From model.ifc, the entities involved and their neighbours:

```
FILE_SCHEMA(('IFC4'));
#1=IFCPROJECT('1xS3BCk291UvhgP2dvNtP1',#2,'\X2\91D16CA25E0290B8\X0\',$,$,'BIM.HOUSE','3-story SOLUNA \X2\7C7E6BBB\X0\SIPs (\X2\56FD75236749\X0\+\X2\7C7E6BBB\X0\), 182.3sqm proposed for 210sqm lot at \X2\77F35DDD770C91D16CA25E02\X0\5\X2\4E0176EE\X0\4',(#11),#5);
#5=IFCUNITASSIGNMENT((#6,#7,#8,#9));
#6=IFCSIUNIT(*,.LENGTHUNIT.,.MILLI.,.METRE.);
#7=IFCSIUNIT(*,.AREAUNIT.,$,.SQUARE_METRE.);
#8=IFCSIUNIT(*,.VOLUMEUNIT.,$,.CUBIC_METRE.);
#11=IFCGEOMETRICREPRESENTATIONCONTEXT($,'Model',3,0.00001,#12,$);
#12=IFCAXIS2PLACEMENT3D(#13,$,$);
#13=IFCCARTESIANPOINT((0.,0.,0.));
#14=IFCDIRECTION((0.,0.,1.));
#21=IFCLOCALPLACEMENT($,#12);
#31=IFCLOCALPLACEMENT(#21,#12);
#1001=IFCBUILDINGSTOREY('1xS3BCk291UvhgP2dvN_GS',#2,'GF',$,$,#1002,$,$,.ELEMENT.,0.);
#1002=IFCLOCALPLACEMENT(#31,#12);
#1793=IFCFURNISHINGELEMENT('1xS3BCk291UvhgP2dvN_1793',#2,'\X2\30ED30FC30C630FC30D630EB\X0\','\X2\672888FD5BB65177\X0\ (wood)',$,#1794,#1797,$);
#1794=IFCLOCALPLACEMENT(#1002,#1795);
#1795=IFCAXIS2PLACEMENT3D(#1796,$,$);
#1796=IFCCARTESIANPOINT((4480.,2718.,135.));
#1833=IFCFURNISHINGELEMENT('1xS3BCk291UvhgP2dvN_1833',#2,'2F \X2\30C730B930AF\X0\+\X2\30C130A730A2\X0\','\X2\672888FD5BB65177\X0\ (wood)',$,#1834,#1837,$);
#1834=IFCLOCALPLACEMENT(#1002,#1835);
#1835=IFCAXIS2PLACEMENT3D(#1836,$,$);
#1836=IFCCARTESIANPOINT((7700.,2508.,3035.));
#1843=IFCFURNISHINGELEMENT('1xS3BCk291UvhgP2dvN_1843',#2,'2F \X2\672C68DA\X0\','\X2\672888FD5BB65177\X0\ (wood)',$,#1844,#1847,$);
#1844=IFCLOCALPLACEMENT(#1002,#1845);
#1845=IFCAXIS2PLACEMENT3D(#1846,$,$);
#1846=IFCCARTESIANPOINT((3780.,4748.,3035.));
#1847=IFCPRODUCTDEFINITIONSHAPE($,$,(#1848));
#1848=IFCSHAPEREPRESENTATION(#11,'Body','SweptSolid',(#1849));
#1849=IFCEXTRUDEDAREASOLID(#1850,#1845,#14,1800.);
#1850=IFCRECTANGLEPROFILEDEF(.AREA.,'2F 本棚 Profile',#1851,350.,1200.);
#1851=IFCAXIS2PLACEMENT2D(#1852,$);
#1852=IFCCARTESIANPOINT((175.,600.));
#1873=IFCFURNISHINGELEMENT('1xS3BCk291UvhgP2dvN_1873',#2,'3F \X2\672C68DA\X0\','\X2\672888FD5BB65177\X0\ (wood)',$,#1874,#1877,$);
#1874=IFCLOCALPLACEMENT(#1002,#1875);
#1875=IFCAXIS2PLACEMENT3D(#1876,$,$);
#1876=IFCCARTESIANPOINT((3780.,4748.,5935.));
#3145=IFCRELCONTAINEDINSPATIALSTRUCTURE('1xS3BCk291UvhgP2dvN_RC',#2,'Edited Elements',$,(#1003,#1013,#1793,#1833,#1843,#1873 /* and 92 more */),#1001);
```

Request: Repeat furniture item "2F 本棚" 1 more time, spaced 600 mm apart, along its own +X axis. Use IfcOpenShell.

```python
import ifcopenshell
import ifcopenshell.api.geometry
import ifcopenshell.api.root
import ifcopenshell.util.element
import ifcopenshell.util.placement

model = ifcopenshell.open("model.ifc")


def reuse_history(source, copy):
    """copy_class also copies each property set's owner history, people and application; keep the originals."""
    for rel in copy.IsDefinedBy:
        if rel.is_a("IfcRelDefinesByProperties") and (history := rel.RelatingPropertyDefinition.OwnerHistory):
            rel.RelatingPropertyDefinition.OwnerHistory = source.OwnerHistory
            ifcopenshell.util.element.remove_deep2(model, history)


source = model.by_id(1843)
base = ifcopenshell.util.placement.get_local_placement(source.ObjectPlacement)
step = base[:3, 0] * 600.0

for i in range(1, 2):
    copy = ifcopenshell.api.root.copy_class(model, product=source)
    copy.Representation = ifcopenshell.util.element.copy_deep(
        model, source.Representation, exclude=["IfcGeometricRepresentationContext", "IfcRepresentationMap"]
    )
    reuse_history(source, copy)
    matrix = base.copy()
    matrix[:3, 3] += i * step
    print("added at", matrix[:3, 3].round(3) + 0.0)
    ifcopenshell.api.geometry.edit_object_placement(model, product=copy, matrix=matrix, is_si=False)

model.write("model_v2.ifc")
```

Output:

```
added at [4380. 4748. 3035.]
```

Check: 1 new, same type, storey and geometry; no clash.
